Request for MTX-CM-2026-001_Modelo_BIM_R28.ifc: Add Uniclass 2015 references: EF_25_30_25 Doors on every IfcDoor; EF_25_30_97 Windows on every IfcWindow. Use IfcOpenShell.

First a look at what the model holds.

```python
import ifcopenshell

model = ifcopenshell.open("MTX-CM-2026-001_Modelo_BIM_R28.ifc")
print(model.schema)
print("classifications:", [c.Name for c in model.by_type("IfcClassification")])
for ifc_class in ("IfcDoor", "IfcRoof", "IfcStair", "IfcWall", "IfcWindow"):
    print(ifc_class, len(model.by_type(ifc_class)))
```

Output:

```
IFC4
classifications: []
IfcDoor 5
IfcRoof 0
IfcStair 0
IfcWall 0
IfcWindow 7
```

```python
import ifcopenshell
import ifcopenshell.api.classification

model = ifcopenshell.open("MTX-CM-2026-001_Modelo_BIM_R28.ifc")

system = ifcopenshell.api.classification.add_classification(model, classification="Uniclass 2015")

codes = {
    "IfcDoor": ("EF_25_30_25", "Doors"),
    "IfcWindow": ("EF_25_30_97", "Windows"),
}
for ifc_class, (code, name) in codes.items():
    products = model.by_type(ifc_class)
    ifcopenshell.api.classification.add_reference(
        model, products=products, classification=system, identification=code, name=name
    )
    print(code, len(products))

model.write("MTX-CM-2026-001_Modelo_BIM_R28_rev.ifc")
```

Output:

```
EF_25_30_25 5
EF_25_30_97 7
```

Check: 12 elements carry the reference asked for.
